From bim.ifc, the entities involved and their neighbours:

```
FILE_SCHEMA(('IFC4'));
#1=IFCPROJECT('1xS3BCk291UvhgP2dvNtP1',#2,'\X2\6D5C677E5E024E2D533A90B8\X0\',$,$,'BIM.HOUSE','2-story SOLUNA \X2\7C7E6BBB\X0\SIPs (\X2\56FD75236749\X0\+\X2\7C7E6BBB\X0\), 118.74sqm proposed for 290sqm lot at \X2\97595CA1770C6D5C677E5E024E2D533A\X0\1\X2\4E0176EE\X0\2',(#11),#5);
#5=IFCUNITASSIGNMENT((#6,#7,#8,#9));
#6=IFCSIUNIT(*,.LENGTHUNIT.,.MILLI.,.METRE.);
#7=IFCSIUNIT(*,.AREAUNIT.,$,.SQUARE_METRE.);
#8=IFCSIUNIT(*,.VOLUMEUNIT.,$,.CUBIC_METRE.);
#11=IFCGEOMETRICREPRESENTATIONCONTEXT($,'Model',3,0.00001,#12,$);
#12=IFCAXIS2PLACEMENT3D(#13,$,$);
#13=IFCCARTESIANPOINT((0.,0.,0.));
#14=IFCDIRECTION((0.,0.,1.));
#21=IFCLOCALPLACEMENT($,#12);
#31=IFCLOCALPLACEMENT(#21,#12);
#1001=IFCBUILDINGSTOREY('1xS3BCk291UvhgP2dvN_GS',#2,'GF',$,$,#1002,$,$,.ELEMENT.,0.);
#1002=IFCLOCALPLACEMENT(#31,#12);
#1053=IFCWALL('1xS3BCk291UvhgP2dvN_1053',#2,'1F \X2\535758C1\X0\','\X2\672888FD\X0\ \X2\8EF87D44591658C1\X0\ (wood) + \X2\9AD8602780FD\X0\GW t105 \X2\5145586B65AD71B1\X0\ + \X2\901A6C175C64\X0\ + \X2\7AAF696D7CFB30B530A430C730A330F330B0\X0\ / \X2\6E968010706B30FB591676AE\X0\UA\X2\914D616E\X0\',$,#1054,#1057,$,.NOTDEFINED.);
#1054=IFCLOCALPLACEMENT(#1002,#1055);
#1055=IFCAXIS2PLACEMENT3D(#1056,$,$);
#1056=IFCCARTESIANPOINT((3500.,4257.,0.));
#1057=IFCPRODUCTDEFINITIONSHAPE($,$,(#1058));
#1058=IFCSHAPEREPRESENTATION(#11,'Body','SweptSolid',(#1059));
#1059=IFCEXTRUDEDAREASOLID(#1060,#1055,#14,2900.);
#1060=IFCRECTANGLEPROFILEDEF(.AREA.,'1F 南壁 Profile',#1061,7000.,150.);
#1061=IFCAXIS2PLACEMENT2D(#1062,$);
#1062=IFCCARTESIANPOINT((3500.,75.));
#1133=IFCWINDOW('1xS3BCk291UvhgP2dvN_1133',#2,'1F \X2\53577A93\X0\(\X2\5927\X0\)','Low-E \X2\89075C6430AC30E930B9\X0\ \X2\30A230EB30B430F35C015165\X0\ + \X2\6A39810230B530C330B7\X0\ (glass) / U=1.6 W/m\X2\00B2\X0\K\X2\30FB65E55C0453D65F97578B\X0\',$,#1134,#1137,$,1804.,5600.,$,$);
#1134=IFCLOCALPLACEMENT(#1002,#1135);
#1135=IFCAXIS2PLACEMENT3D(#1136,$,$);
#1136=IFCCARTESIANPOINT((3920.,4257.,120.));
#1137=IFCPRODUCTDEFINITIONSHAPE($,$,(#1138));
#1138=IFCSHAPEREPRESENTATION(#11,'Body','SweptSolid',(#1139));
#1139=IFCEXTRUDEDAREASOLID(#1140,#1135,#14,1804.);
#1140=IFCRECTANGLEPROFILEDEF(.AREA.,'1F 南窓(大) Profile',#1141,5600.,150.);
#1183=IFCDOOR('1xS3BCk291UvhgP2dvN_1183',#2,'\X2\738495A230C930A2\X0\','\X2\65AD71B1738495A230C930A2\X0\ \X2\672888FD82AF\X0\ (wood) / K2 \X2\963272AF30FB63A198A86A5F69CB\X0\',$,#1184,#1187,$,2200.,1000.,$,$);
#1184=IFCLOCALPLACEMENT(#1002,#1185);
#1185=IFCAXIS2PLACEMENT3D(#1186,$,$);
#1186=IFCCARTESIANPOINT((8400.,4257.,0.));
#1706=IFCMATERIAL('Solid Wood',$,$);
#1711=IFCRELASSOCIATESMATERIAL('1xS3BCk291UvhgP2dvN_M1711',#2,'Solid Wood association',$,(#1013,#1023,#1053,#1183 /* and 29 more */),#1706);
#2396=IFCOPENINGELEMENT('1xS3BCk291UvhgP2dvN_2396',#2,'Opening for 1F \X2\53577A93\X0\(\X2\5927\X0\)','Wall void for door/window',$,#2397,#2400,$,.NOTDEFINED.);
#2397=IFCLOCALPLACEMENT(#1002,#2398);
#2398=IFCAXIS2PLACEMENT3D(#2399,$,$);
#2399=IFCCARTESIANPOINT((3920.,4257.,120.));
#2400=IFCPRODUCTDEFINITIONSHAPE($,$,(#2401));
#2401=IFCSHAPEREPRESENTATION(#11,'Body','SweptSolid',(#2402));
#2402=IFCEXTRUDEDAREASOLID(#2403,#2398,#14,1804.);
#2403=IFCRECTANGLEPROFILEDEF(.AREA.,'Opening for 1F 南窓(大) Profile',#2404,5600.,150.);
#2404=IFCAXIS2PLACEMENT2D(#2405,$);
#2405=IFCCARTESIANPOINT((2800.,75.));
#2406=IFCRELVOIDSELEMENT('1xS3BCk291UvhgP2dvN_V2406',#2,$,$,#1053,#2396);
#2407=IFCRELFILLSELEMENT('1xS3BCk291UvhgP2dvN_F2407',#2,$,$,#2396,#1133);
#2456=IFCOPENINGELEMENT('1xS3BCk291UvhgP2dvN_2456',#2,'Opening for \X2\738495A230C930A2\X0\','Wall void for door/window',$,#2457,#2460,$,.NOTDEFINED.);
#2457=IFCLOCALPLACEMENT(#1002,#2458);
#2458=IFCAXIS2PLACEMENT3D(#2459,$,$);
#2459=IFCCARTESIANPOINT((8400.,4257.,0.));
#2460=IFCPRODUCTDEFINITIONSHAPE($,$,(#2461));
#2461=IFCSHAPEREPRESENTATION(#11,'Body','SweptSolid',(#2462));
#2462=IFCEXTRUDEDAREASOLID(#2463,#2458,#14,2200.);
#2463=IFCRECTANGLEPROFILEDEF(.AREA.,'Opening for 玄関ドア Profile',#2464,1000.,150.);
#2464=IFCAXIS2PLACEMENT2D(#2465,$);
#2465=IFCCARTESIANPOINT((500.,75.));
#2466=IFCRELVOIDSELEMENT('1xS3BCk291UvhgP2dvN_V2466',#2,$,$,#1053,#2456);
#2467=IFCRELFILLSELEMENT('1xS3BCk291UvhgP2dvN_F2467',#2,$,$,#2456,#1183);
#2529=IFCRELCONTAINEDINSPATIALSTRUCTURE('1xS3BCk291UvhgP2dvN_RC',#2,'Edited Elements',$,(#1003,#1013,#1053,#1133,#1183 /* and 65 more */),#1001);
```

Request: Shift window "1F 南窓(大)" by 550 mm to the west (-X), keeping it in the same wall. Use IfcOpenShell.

```python
import ifcopenshell
import ifcopenshell.api.geometry
import ifcopenshell.util.placement

model = ifcopenshell.open("bim.ifc")

window = model.by_guid("1xS3BCk291UvhgP2dvN_1133")
opening = window.FillsVoids[0].RelatingOpeningElement
wall = opening.VoidsElements[0].RelatingBuildingElement

wall_matrix = ifcopenshell.util.placement.get_local_placement(wall.ObjectPlacement)
shift = wall_matrix[:3, 0] * -550.0
before = ifcopenshell.util.placement.get_local_placement(window.ObjectPlacement)[:3, 3].copy()

# The window is not placed relative to its opening, so move both.
for product in (opening, window):
    matrix = ifcopenshell.util.placement.get_local_placement(product.ObjectPlacement)
    matrix[:3, 3] += shift
    ifcopenshell.api.geometry.edit_object_placement(model, product=product, matrix=matrix, is_si=False)

after = ifcopenshell.util.placement.get_local_placement(window.ObjectPlacement)[:3, 3]
print("window moved by", (after - before).round(3) + 0.0)

model.write("bim_rev.ifc")
```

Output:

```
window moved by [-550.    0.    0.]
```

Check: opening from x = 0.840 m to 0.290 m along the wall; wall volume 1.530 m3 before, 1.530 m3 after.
